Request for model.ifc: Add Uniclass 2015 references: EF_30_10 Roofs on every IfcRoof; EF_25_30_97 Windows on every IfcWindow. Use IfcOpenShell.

First a look at what the model holds.

```python
import ifcopenshell

model = ifcopenshell.open("model.ifc")
print(model.schema)
print("classifications:", [c.Name for c in model.by_type("IfcClassification")])
for ifc_class in ("IfcDoor", "IfcRoof", "IfcStair", "IfcWall", "IfcWindow"):
    print(ifc_class, len(model.by_type(ifc_class)))
```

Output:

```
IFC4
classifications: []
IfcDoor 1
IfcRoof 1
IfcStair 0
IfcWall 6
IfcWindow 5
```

```python
import ifcopenshell
import ifcopenshell.api.classification

model = ifcopenshell.open("model.ifc")

system = ifcopenshell.api.classification.add_classification(model, classification="Uniclass 2015")

codes = {
    "IfcRoof": ("EF_30_10", "Roofs"),
    "IfcWindow": ("EF_25_30_97", "Windows"),
}
for ifc_class, (code, name) in codes.items():
    products = model.by_type(ifc_class)
    ifcopenshell.api.classification.add_reference(
        model, products=products, classification=system, identification=code, name=name
    )
    print(code, len(products))

model.write("model-out.ifc")
```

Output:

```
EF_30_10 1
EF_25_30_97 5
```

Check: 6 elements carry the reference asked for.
